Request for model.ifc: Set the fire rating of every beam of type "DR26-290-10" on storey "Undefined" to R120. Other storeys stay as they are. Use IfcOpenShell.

First a look at what the model holds.

```python
import ifcopenshell
import ifcopenshell.util.element

model = ifcopenshell.open("model.ifc")
print(model.schema)
storey = next(s for s in model.by_type("IfcBuildingStorey") if s.Name == "Undefined")
beams = [e for e in ifcopenshell.util.element.get_decomposition(storey) if e.is_a("IfcBeam")]
seen = {}
for e in beams:
    element_type = ifcopenshell.util.element.get_type(e)
    key = (element_type.Name if element_type != e and element_type else None, ifcopenshell.util.element.get_pset(e, "Pset_BeamCommon", "FireRating"))
    seen[key] = seen.get(key, 0) + 1
for (name, value), count in sorted(seen.items(), key=str):
    print(count, "x", name, "|", value)
```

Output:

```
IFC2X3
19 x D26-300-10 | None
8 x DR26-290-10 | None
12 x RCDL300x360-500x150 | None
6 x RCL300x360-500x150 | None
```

```python
import ifcopenshell
import ifcopenshell.api.pset
import ifcopenshell.util.element

model = ifcopenshell.open("model.ifc")

storey = next(s for s in model.by_type("IfcBuildingStorey") if s.Name == "Undefined")
beams = [e for e in ifcopenshell.util.element.get_decomposition(storey) if e.is_a("IfcBeam")]

count = 0
for e in beams:
    element_type = ifcopenshell.util.element.get_type(e)
    if element_type in (None, e) or element_type.Name != "DR26-290-10":
        continue
    found = ifcopenshell.util.element.get_pset(e, "Pset_BeamCommon", should_inherit=False)
    if found:
        pset = model.by_id(found["id"])
        if len(ifcopenshell.util.element.get_elements_by_pset(pset)) > 1:
            pset = ifcopenshell.api.pset.unshare_pset(model, products=[e], pset=pset)[0]
    else:
        pset = ifcopenshell.api.pset.add_pset(model, product=e, name="Pset_BeamCommon")
    ifcopenshell.api.pset.edit_pset(model, pset=pset, properties={"FireRating": "R120"})
    count += 1

print(count, "beams updated")

model.write("model-out.ifc")
```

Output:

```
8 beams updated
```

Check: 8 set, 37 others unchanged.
